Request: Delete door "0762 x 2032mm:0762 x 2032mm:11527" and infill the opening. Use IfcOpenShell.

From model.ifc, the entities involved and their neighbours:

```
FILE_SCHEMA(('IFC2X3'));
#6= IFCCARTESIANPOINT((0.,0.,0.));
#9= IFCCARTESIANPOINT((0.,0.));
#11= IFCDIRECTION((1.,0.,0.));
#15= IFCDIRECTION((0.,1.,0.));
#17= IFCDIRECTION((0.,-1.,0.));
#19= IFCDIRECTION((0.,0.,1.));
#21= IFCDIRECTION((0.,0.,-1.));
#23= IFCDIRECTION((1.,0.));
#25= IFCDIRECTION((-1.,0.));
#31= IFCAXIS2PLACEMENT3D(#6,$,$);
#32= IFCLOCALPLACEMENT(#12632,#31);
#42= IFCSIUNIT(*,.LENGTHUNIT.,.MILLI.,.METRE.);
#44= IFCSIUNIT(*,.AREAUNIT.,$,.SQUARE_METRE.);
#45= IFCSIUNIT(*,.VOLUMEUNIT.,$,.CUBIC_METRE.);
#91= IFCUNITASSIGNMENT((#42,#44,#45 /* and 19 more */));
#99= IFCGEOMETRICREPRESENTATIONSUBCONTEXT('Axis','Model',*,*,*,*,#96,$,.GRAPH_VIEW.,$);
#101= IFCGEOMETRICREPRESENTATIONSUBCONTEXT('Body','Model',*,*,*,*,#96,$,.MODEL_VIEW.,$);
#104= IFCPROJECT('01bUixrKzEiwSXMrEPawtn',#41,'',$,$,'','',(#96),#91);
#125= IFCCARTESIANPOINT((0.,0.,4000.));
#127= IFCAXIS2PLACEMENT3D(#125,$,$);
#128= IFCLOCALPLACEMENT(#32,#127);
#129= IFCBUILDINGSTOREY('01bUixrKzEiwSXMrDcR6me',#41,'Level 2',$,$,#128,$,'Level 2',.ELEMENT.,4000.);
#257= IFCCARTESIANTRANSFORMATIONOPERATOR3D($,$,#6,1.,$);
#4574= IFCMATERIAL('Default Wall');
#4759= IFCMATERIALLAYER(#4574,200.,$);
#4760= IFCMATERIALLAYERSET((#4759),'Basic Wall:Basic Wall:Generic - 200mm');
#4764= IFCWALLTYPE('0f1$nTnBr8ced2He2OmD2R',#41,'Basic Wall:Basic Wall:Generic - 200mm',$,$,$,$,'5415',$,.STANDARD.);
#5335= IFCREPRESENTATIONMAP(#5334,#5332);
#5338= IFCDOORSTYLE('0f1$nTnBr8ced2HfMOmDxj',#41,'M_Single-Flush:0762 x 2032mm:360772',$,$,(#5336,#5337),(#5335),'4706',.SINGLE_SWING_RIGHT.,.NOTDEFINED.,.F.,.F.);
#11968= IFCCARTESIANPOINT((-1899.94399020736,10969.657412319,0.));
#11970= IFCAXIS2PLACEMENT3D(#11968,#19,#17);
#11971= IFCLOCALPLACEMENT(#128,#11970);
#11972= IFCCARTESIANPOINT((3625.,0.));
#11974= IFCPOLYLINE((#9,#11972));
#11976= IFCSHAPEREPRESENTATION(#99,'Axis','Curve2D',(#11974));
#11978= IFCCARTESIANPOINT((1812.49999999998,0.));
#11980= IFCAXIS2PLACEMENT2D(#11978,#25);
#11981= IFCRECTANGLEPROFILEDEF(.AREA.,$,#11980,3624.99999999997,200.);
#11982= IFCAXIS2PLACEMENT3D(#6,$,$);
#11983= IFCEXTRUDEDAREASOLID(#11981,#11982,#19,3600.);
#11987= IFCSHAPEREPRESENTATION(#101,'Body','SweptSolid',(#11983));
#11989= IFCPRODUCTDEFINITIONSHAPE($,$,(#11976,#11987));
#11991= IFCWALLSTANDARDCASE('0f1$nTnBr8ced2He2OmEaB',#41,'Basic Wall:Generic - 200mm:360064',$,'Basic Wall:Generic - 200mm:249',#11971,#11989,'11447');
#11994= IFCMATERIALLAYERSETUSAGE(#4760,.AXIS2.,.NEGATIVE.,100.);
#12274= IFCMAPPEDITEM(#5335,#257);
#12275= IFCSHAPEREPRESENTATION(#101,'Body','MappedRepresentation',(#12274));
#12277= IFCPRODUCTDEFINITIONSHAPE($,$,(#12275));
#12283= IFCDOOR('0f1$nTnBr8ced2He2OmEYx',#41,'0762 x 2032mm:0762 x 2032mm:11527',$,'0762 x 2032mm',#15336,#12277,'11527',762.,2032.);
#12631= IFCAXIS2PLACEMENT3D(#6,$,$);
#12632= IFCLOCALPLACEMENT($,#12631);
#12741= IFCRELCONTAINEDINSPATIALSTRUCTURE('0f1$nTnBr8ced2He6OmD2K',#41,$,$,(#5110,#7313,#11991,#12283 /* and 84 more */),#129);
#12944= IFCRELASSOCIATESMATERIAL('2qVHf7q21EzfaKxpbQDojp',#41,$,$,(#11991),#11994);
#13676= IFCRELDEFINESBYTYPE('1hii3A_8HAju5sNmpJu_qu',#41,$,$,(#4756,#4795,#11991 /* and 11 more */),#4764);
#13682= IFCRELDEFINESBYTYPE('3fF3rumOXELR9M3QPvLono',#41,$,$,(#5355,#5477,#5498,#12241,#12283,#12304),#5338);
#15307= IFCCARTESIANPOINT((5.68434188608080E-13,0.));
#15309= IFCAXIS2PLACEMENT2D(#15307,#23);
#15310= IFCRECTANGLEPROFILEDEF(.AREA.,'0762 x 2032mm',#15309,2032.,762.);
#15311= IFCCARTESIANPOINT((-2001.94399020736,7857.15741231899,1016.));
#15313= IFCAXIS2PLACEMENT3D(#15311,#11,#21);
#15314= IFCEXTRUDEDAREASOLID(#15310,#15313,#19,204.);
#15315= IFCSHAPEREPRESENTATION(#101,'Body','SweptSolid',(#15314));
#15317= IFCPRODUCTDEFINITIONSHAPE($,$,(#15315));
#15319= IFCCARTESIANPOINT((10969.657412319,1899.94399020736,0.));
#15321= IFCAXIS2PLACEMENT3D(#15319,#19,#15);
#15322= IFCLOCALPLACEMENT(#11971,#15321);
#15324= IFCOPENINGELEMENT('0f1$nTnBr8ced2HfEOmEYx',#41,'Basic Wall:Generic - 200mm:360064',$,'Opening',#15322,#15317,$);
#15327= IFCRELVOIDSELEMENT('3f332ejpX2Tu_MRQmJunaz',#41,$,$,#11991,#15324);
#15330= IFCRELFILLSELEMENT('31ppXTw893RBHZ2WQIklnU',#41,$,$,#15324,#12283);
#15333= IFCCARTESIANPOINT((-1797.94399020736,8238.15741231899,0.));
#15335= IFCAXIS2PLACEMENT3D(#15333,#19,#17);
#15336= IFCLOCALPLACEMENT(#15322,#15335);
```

```python
import ifcopenshell
import ifcopenshell.api.feature
import ifcopenshell.api.root
import ifcopenshell.geom
import ifcopenshell.util.shape

model = ifcopenshell.open("model.ifc")
settings = ifcopenshell.geom.settings()


def volume(element):
    """Net volume in cubic metres, openings subtracted."""
    shape = ifcopenshell.geom.create_shape(settings, element)
    return ifcopenshell.util.shape.get_volume(shape.geometry)


door = model.by_guid("0f1$nTnBr8ced2He2OmEYx")
opening = door.FillsVoids[0].RelatingOpeningElement
wall = opening.VoidsElements[0].RelatingBuildingElement
before = volume(wall)

ifcopenshell.api.root.remove_product(model, product=door)
ifcopenshell.api.feature.remove_feature(model, feature=opening)

after = volume(wall)

print(f"wall volume {before:.3f} -> {after:.3f} m3")

model.write("model_v2.ifc")
```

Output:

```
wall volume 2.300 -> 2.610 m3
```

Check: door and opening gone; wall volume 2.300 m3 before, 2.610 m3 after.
